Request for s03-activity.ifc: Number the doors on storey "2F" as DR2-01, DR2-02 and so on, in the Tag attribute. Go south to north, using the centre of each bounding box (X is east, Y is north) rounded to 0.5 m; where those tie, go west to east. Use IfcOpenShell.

First a look at what the model holds.

```python
import ifcopenshell
import ifcopenshell.util.element
import ifcopenshell.util.placement

model = ifcopenshell.open("s03-activity.ifc")
print(model.schema)
storey = next(s for s in model.by_type("IfcBuildingStorey") if s.Name == "2F")
doors = [e for e in ifcopenshell.util.element.get_decomposition(storey) if e.is_a("IfcDoor")]
for e in sorted(doors, key=lambda e: e.id()):
    origin = ifcopenshell.util.placement.get_local_placement(e.ObjectPlacement)[:3, 3]
    print(e.id(), e.Tag, e.Name, origin.round(2) + 0.0, sep=" | ")
```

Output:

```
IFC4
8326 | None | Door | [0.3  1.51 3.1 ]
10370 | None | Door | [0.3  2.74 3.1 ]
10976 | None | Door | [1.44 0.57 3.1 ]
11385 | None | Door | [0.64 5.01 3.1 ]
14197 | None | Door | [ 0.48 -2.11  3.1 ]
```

```python
import ifcopenshell
import ifcopenshell.geom
import ifcopenshell.util.element
import ifcopenshell.util.shape

model = ifcopenshell.open("s03-activity.ifc")
settings = ifcopenshell.geom.settings()
settings.set("use-world-coords", True)


def centre(element):
    shape = ifcopenshell.geom.create_shape(settings, element)
    return ifcopenshell.util.shape.get_bbox_centroid(shape.geometry)


storey = next(s for s in model.by_type("IfcBuildingStorey") if s.Name == "2F")
doors = [e for e in ifcopenshell.util.element.get_decomposition(storey) if e.is_a("IfcDoor")]

# Insertion points can sit at a corner or the storey origin, so sort by the geometry (in metres).
centres = {e: centre(e) for e in doors}
doors.sort(key=lambda e: (round(centres[e][1] / 0.5), centres[e][0]))

for i, e in enumerate(doors, start=1):
    number = f"DR2-{i:02d}"
    e.Tag = number
    print(e.id(), number)

model.write("s03-activity_v2.ifc")
```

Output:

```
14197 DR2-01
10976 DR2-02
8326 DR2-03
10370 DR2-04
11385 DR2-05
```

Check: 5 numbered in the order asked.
